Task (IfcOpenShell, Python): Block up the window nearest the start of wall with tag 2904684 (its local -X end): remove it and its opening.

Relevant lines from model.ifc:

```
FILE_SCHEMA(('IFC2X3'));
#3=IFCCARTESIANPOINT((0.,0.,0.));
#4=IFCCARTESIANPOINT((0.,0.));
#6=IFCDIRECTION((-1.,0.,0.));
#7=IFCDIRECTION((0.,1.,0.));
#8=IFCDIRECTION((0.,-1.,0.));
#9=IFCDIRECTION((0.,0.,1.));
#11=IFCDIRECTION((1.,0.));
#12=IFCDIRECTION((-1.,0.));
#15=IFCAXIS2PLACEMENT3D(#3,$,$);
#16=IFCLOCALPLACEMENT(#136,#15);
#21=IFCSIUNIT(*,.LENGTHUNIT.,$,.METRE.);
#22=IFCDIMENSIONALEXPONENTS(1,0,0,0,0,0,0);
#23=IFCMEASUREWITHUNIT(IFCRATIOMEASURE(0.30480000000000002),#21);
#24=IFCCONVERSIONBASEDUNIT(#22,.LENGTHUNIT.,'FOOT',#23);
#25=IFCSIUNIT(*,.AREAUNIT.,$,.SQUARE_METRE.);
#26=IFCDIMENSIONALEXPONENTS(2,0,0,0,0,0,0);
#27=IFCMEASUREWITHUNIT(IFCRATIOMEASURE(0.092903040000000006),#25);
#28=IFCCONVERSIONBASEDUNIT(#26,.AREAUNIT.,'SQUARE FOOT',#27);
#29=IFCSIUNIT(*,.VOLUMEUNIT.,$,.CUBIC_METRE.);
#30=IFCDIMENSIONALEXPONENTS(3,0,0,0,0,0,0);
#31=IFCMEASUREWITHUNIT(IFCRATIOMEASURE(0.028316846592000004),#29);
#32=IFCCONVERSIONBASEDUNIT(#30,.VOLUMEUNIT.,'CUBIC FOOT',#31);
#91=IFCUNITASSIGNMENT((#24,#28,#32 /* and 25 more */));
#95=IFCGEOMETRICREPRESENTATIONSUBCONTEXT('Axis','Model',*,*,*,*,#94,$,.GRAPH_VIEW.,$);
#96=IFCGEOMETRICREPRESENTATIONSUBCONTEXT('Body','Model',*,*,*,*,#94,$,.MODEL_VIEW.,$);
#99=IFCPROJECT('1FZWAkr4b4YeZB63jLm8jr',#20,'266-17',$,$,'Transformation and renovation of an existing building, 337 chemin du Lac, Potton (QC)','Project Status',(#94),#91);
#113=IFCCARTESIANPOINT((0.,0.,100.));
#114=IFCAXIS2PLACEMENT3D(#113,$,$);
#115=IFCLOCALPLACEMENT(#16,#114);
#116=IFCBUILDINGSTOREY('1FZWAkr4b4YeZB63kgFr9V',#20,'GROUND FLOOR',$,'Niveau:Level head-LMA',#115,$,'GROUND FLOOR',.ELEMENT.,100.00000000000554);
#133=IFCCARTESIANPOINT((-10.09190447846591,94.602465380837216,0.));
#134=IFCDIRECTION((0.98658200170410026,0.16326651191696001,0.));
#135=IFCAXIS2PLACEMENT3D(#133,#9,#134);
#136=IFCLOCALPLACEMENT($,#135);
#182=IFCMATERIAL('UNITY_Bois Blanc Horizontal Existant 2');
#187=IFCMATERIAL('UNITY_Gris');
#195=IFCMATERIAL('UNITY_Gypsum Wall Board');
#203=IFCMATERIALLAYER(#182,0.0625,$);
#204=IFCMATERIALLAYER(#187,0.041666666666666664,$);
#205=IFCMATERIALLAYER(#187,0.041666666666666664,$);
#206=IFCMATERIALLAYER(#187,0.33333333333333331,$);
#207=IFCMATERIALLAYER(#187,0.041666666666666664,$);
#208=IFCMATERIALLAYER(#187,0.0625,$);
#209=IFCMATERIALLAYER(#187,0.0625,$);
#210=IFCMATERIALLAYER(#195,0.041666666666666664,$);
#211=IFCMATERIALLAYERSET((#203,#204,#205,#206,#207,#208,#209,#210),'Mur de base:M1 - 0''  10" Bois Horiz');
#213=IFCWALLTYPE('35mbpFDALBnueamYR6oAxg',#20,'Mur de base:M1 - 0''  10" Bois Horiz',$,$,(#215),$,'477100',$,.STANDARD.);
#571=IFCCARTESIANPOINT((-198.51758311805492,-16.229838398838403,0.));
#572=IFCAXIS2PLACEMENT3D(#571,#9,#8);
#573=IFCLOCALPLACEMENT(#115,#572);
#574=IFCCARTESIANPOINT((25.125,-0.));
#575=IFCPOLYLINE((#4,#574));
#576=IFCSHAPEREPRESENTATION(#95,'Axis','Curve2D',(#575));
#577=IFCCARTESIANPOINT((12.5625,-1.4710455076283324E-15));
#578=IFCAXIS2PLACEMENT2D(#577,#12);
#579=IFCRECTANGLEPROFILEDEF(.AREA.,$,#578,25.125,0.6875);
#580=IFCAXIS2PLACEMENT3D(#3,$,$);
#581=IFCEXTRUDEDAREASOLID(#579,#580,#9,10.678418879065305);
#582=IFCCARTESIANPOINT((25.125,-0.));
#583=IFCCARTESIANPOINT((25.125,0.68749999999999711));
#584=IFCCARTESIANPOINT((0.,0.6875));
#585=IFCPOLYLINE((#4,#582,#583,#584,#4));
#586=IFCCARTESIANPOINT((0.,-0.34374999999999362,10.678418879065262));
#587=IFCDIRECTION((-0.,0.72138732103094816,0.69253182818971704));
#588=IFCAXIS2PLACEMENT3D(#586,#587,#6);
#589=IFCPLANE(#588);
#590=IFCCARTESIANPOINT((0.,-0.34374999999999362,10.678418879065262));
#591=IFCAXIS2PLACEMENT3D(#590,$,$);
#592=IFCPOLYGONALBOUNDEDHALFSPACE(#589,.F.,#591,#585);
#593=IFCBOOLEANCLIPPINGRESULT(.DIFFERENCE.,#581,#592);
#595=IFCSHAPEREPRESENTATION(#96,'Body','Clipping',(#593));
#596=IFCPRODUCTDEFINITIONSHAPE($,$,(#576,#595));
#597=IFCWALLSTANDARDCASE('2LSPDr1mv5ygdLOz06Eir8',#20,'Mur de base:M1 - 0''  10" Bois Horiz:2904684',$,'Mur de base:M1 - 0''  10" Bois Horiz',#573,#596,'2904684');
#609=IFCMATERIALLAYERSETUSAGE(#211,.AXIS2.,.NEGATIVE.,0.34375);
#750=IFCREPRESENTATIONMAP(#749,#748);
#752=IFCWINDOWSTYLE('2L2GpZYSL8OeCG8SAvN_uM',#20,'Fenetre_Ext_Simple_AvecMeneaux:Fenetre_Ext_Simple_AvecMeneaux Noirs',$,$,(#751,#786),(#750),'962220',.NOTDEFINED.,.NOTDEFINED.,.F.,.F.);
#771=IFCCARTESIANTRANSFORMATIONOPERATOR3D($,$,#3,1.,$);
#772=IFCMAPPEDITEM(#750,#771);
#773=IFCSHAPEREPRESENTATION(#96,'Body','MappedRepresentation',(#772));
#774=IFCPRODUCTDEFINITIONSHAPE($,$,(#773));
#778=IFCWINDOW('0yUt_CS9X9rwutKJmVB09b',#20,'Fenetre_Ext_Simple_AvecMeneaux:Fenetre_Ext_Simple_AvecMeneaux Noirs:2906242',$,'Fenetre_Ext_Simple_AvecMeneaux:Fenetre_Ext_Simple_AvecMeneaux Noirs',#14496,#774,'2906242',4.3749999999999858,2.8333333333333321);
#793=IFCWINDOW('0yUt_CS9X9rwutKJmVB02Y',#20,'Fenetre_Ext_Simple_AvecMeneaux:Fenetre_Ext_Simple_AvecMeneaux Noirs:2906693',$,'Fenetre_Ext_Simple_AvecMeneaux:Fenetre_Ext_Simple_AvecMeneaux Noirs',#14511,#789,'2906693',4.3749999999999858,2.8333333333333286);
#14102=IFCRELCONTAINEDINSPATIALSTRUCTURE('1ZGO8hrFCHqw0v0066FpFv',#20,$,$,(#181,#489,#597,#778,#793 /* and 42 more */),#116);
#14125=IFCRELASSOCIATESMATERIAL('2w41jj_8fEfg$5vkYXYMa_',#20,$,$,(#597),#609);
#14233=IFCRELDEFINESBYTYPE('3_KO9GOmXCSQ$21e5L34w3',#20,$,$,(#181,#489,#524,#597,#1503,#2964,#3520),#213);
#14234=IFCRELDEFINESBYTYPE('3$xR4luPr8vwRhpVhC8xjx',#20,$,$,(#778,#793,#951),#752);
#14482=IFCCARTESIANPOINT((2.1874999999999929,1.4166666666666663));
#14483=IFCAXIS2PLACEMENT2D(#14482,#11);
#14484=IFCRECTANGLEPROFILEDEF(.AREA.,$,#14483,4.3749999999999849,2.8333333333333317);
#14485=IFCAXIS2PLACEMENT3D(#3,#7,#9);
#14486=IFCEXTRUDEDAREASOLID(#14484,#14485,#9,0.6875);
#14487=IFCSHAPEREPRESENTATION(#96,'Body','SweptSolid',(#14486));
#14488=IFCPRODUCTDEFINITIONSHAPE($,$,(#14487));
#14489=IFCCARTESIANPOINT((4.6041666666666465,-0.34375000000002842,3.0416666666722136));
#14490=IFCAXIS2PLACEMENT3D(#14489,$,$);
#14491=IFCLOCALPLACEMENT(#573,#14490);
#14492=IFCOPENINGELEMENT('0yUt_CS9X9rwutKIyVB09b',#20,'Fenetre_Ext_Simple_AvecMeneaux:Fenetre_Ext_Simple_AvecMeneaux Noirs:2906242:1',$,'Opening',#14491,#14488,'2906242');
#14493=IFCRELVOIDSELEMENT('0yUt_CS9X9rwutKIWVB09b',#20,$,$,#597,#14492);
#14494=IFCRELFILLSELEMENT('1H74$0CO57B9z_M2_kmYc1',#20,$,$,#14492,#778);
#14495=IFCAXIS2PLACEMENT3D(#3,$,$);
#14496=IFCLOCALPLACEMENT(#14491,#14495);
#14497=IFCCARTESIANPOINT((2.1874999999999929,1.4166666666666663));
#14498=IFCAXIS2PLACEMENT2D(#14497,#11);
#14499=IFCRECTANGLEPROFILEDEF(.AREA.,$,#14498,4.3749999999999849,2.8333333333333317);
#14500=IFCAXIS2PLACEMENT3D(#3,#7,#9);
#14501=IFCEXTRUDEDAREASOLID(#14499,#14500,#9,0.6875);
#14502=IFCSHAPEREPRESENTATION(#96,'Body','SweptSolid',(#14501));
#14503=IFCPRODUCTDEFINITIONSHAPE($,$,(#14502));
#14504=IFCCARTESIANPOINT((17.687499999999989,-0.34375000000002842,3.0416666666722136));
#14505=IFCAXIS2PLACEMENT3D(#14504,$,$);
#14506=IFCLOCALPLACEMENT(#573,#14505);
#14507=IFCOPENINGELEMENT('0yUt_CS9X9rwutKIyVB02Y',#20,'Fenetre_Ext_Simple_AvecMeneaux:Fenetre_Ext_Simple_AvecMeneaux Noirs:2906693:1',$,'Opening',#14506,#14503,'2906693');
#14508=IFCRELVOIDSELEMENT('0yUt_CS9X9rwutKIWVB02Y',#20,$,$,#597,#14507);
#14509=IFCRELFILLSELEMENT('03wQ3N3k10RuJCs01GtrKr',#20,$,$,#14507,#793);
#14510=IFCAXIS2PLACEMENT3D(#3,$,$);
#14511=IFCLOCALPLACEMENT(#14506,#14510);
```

```python
import ifcopenshell
import ifcopenshell.api.feature
import ifcopenshell.api.root
import ifcopenshell.geom
import ifcopenshell.util.shape

model = ifcopenshell.open("model.ifc")
settings = ifcopenshell.geom.settings()


def volume(element):
    """Net volume in cubic metres, openings subtracted."""
    shape = ifcopenshell.geom.create_shape(settings, element)
    return ifcopenshell.util.shape.get_volume(shape.geometry)


window = model.by_id(778)
opening = window.FillsVoids[0].RelatingOpeningElement
wall = opening.VoidsElements[0].RelatingBuildingElement
before = volume(wall)

ifcopenshell.api.root.remove_product(model, product=window)
ifcopenshell.api.feature.remove_feature(model, feature=opening)

after = volume(wall)

print(f"wall volume {before:.3f} -> {after:.3f} m3")

model.write("model_rev.ifc")
```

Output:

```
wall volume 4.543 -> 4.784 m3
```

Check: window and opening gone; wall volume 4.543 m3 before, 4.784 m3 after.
